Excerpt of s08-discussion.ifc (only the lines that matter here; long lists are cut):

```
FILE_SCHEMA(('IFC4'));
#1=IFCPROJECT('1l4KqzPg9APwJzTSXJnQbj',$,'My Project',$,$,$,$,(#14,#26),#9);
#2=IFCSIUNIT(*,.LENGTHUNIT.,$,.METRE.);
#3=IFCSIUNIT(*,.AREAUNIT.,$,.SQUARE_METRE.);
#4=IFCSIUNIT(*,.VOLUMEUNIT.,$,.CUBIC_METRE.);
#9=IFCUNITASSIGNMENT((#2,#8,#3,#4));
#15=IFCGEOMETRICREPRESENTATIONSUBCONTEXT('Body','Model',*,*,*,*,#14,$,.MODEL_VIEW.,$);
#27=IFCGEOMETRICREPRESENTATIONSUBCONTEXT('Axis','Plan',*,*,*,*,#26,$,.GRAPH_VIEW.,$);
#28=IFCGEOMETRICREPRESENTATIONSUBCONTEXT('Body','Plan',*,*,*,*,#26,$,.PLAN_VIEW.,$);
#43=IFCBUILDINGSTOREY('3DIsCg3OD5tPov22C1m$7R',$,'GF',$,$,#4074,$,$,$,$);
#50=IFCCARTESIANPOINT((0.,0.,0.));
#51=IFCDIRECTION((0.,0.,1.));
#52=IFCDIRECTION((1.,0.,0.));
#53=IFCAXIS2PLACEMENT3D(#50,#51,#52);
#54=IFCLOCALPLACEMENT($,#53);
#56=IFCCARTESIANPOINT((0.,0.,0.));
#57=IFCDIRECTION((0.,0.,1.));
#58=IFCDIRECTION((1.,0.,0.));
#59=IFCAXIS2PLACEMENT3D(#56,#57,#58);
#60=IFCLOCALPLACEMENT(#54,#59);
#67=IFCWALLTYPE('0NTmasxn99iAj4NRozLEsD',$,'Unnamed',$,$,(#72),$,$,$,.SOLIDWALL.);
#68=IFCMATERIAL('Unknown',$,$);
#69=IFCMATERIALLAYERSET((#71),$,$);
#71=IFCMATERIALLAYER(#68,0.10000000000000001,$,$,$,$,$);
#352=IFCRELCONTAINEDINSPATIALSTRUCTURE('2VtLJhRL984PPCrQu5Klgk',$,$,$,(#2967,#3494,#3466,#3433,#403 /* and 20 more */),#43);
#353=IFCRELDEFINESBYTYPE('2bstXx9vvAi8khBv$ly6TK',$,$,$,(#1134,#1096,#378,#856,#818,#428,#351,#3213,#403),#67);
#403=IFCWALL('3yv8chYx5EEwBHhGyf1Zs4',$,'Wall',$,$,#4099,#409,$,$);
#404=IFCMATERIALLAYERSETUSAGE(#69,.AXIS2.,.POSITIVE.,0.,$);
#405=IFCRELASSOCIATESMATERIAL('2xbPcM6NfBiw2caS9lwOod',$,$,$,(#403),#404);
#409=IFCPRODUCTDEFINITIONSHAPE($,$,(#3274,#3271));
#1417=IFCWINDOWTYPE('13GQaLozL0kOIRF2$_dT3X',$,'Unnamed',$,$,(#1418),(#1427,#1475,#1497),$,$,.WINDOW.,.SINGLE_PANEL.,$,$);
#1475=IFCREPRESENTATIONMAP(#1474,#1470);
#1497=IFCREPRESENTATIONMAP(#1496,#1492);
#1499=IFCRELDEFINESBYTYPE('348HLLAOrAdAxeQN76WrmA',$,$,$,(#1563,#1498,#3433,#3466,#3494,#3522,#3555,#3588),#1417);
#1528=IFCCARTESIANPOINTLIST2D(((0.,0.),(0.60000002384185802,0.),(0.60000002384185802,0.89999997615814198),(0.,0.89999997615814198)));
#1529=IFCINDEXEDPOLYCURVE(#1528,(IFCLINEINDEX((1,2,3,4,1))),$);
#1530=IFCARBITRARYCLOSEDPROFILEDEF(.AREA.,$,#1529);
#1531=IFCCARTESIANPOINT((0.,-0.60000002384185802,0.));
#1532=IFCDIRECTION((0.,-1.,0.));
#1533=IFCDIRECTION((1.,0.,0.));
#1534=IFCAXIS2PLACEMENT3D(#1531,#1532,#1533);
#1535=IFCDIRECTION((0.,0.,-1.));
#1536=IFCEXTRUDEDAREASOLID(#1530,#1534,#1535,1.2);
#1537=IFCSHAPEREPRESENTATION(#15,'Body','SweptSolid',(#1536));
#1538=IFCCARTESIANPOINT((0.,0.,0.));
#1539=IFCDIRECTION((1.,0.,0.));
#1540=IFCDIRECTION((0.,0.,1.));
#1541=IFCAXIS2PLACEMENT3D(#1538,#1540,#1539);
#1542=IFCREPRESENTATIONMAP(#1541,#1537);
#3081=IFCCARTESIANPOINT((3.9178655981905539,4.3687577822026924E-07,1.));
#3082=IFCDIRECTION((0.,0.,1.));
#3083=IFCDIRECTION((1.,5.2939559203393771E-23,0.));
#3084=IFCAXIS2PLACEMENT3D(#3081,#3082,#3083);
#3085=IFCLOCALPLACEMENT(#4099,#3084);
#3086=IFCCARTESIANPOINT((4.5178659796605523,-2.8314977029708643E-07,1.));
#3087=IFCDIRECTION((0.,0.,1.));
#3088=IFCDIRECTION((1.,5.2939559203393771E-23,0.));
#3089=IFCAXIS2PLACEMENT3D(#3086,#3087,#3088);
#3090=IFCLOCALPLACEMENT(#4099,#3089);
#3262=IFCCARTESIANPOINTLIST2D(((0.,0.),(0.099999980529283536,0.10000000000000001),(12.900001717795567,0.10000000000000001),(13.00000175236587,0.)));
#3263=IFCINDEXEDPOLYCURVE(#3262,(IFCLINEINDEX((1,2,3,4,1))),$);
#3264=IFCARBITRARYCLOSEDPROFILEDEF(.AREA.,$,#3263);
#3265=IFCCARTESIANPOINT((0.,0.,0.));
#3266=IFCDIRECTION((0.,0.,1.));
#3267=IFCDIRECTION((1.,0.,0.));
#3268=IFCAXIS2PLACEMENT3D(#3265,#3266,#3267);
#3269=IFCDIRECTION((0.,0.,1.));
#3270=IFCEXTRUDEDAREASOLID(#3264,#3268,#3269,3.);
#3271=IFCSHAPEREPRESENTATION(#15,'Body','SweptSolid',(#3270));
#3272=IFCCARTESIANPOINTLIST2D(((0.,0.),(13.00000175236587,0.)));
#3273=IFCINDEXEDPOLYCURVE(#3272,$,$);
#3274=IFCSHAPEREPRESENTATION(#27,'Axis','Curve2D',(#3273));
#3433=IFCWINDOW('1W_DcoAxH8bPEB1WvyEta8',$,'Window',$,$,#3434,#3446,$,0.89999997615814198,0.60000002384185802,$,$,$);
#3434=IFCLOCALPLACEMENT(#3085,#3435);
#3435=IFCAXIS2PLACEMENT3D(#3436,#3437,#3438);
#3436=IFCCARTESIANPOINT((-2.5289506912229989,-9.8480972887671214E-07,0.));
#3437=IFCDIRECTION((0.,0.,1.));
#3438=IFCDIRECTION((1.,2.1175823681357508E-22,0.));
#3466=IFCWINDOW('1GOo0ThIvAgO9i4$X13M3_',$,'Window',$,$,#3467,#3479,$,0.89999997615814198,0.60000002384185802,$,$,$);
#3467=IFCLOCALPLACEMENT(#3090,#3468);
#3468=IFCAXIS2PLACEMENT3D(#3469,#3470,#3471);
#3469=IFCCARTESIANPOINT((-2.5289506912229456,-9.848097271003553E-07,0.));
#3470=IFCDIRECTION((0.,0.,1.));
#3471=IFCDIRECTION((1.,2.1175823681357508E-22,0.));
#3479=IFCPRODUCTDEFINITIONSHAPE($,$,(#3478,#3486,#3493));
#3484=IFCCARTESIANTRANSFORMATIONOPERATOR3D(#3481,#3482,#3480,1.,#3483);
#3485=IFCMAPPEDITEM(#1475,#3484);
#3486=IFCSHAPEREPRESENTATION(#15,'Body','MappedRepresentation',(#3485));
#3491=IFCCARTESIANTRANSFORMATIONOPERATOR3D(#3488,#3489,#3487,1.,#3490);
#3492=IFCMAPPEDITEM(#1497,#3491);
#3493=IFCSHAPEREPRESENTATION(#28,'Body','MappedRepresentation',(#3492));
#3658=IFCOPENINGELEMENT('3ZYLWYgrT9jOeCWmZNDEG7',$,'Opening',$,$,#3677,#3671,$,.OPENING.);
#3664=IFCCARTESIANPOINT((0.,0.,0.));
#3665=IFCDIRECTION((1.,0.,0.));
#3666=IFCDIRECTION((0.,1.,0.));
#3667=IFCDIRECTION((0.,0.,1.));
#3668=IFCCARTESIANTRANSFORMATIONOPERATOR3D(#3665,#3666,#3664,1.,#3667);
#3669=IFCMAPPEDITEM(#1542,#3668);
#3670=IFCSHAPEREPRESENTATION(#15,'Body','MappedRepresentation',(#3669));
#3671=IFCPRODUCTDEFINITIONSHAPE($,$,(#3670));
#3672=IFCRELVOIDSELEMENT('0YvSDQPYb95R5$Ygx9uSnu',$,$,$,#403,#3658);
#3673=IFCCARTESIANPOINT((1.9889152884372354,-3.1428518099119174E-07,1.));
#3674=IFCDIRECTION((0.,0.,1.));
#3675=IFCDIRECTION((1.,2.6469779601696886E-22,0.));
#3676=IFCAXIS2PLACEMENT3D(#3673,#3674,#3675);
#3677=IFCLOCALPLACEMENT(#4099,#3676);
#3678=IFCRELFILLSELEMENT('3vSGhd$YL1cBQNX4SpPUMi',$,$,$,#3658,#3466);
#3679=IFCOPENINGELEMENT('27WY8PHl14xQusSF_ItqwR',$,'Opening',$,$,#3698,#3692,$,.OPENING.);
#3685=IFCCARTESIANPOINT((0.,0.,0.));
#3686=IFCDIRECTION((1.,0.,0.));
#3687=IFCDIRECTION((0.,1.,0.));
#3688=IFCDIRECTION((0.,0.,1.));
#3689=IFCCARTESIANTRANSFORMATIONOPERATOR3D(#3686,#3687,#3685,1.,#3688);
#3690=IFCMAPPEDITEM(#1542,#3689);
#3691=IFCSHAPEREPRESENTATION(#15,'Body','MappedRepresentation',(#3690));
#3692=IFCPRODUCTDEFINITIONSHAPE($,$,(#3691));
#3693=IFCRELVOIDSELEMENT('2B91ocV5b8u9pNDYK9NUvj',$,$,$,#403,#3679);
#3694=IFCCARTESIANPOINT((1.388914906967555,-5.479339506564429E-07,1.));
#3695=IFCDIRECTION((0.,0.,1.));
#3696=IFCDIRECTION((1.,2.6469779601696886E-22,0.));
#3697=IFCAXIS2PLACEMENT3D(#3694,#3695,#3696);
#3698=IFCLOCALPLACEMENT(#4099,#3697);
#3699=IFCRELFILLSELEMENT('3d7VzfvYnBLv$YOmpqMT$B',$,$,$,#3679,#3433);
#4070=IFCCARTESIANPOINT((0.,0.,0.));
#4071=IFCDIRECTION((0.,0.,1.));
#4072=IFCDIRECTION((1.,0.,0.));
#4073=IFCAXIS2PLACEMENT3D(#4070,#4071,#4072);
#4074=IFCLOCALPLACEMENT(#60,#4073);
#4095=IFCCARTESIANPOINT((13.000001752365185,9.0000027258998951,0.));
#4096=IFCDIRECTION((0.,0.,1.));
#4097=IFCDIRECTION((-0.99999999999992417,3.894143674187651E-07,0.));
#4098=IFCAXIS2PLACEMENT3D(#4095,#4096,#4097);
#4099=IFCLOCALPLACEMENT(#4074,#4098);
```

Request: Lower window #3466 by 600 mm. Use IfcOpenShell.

```python
import numpy as np
import ifcopenshell
import ifcopenshell.api.geometry
import ifcopenshell.util.placement
import ifcopenshell.util.unit

model = ifcopenshell.open("s08-discussion.ifc")
unit_scale = ifcopenshell.util.unit.calculate_unit_scale(model)

window = model.by_guid("1GOo0ThIvAgO9i4$X13M3_")
opening = window.FillsVoids[0].RelatingOpeningElement
dz = -0.6

shift = np.array([0.0, 0.0, dz])
# The window is not placed relative to its opening, so move both.
for product in (opening, window):
    matrix = ifcopenshell.util.placement.get_local_placement(product.ObjectPlacement)
    matrix[:3, 3] += shift
    ifcopenshell.api.geometry.edit_object_placement(model, product=product, matrix=matrix, is_si=False)

print(f"moved by {dz * unit_scale:+.3f} m")

model.write("s08-discussion_rev.ifc")
```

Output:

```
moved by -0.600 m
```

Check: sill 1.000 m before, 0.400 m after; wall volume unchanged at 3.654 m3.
